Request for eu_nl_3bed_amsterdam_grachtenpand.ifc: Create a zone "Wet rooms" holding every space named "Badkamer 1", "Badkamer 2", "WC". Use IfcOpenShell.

First a look at what the model holds.

```python
import ifcopenshell

model = ifcopenshell.open("eu_nl_3bed_amsterdam_grachtenpand.ifc")
print(model.schema)
seen = {}
for space in model.by_type("IfcSpace"):
    seen[space.LongName] = seen.get(space.LongName, 0) + 1
for name, count in sorted(seen.items(), key=str):
    print(count, "x", name)
print("zones:", [z.Name for z in model.by_type("IfcZone")][:20])
```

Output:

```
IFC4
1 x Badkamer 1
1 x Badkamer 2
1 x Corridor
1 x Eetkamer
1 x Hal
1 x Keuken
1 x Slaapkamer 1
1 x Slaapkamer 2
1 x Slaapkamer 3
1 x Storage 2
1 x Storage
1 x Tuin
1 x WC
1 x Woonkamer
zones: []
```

```python
import ifcopenshell
import ifcopenshell.api.group
import ifcopenshell.api.root

model = ifcopenshell.open("eu_nl_3bed_amsterdam_grachtenpand.ifc")

names = {"Badkamer 1", "Badkamer 2", "WC"}
spaces = [s for s in model.by_type("IfcSpace") if s.LongName in names]

zone = ifcopenshell.api.root.create_entity(model, ifc_class="IfcZone", name="Wet rooms")
ifcopenshell.api.group.assign_group(model, products=spaces, group=zone)
print(len(spaces), "spaces in", zone.Name)

model.write("eu_nl_3bed_amsterdam_grachtenpand_updated.ifc")
```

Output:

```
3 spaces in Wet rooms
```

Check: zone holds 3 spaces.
